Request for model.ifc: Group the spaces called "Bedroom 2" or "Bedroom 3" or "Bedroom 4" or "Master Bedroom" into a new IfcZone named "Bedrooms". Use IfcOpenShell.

First a look at what the model holds.

```python
import ifcopenshell

model = ifcopenshell.open("model.ifc")
print(model.schema)
seen = {}
for space in model.by_type("IfcSpace"):
    seen[space.LongName] = seen.get(space.LongName, 0) + 1
for name, count in sorted(seen.items(), key=str):
    print(count, "x", name)
print("zones:", [z.Name for z in model.by_type("IfcZone")][:20])
```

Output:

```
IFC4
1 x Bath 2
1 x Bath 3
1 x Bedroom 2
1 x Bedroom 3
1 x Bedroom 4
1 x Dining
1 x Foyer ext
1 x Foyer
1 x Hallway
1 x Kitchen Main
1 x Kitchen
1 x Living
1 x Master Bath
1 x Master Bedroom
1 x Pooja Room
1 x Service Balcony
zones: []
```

```python
import ifcopenshell
import ifcopenshell.api.group
import ifcopenshell.api.root

model = ifcopenshell.open("model.ifc")

names = {"Bedroom 2", "Bedroom 3", "Bedroom 4", "Master Bedroom"}
spaces = [s for s in model.by_type("IfcSpace") if s.LongName in names]

zone = ifcopenshell.api.root.create_entity(model, ifc_class="IfcZone", name="Bedrooms")
ifcopenshell.api.group.assign_group(model, products=spaces, group=zone)
print(len(spaces), "spaces in", zone.Name)

model.write("model_v2.ifc")
```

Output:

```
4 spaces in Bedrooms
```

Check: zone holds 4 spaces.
